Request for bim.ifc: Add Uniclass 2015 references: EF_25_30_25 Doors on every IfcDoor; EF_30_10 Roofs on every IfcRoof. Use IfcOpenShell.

First a look at what the model holds.

```python
import ifcopenshell

model = ifcopenshell.open("bim.ifc")
print(model.schema)
print("classifications:", [c.Name for c in model.by_type("IfcClassification")])
for ifc_class in ("IfcDoor", "IfcRoof", "IfcStair", "IfcWall", "IfcWindow"):
    print(ifc_class, len(model.by_type(ifc_class)))
```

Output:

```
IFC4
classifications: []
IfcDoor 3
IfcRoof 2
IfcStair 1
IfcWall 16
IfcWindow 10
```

```python
import ifcopenshell
import ifcopenshell.api.classification

model = ifcopenshell.open("bim.ifc")

system = ifcopenshell.api.classification.add_classification(model, classification="Uniclass 2015")

codes = {
    "IfcDoor": ("EF_25_30_25", "Doors"),
    "IfcRoof": ("EF_30_10", "Roofs"),
}
for ifc_class, (code, name) in codes.items():
    products = model.by_type(ifc_class)
    ifcopenshell.api.classification.add_reference(
        model, products=products, classification=system, identification=code, name=name
    )
    print(code, len(products))

model.write("bim_rev.ifc")
```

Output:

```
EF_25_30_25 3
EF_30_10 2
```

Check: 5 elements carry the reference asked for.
